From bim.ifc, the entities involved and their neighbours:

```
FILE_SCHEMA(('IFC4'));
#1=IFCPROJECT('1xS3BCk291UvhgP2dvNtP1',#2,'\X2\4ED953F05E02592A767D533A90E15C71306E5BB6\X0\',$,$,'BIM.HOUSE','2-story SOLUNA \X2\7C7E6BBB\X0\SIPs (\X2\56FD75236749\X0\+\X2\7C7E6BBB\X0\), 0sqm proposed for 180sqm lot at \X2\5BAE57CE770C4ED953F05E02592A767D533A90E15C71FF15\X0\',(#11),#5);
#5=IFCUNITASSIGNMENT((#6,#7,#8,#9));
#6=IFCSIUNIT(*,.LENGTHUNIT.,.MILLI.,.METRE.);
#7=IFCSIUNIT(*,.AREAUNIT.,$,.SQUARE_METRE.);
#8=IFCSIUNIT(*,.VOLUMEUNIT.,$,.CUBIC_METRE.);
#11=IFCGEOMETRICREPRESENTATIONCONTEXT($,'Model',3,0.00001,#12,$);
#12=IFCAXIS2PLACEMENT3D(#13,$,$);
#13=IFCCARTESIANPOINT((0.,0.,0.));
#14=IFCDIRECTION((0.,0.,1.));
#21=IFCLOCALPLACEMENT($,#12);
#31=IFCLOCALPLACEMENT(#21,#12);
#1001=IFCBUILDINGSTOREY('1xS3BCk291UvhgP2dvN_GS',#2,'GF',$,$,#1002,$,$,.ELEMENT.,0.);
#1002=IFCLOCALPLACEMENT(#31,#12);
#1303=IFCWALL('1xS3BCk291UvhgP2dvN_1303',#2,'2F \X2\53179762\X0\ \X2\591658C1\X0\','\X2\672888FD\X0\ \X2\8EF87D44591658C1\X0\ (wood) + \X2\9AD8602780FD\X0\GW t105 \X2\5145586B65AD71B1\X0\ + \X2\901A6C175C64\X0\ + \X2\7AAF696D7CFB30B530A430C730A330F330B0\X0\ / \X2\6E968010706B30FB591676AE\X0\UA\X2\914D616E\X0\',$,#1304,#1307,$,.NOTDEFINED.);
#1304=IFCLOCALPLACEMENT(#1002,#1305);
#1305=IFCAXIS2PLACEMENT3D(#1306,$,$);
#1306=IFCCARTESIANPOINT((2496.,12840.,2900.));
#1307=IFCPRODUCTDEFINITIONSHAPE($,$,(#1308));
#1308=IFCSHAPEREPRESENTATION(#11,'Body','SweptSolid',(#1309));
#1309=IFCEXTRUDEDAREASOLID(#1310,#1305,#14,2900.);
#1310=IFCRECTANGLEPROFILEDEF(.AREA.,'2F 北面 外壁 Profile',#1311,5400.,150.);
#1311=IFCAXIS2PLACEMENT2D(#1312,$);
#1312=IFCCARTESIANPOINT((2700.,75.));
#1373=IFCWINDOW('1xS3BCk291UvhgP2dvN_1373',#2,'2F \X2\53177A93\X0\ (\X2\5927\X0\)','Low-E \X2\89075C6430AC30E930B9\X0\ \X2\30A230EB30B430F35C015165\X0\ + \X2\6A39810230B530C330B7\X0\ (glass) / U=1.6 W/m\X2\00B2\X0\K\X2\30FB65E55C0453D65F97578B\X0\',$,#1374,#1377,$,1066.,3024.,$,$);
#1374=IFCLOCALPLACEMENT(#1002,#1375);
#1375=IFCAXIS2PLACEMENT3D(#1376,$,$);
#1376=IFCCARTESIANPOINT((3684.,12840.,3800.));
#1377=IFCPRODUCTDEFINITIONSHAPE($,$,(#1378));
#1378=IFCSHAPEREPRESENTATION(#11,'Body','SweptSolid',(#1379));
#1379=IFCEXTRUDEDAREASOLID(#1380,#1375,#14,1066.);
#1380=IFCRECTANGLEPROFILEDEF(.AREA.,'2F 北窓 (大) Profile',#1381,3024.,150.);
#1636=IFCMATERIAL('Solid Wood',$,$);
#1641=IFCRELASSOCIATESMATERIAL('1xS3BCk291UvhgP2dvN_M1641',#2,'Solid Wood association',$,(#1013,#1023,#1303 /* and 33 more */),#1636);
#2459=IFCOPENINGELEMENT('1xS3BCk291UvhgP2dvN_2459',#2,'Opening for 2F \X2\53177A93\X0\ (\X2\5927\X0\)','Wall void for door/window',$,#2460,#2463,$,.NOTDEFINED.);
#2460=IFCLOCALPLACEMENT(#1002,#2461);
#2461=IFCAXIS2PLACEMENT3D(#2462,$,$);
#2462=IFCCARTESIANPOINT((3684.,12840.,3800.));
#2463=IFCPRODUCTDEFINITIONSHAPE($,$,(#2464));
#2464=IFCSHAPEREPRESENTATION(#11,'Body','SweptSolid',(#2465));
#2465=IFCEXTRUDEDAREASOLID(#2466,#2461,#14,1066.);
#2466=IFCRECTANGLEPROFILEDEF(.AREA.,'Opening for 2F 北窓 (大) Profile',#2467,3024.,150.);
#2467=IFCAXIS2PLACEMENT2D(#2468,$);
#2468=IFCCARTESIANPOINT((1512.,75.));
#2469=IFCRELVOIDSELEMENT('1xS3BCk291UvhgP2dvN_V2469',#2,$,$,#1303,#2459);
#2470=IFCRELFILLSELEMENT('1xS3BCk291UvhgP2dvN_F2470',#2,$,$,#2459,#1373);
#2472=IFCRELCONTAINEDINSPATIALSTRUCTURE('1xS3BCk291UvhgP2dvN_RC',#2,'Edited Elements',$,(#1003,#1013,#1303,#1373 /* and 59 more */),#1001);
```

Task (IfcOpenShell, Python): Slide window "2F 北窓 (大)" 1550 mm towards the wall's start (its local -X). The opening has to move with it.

```python
import ifcopenshell
import ifcopenshell.api.geometry
import ifcopenshell.util.placement
import ifcopenshell.util.unit

model = ifcopenshell.open("bim.ifc")
unit_scale = ifcopenshell.util.unit.calculate_unit_scale(model)

window = model.by_guid("1xS3BCk291UvhgP2dvN_1373")
opening = window.FillsVoids[0].RelatingOpeningElement
wall = opening.VoidsElements[0].RelatingBuildingElement

wall_matrix = ifcopenshell.util.placement.get_local_placement(wall.ObjectPlacement)
shift = wall_matrix[:3, 0] * -1.55 / unit_scale
before = ifcopenshell.util.placement.get_local_placement(window.ObjectPlacement)[:3, 3].copy()

# The window is not placed relative to its opening, so move both.
for product in (opening, window):
    matrix = ifcopenshell.util.placement.get_local_placement(product.ObjectPlacement)
    matrix[:3, 3] += shift
    ifcopenshell.api.geometry.edit_object_placement(model, product=product, matrix=matrix, is_si=False)

after = ifcopenshell.util.placement.get_local_placement(window.ObjectPlacement)[:3, 3]
print("window moved by", (after - before).round(3) + 0.0)

model.write("bim-out.ifc")
```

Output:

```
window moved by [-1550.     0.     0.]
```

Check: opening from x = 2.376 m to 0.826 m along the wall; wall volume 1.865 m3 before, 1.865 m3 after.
